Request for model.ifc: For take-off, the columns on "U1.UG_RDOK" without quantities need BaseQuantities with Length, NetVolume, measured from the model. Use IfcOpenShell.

First a look at what the model holds.

```python
import ifcopenshell
import ifcopenshell.util.element
import ifcopenshell.util.unit

model = ifcopenshell.open("model.ifc")
print(model.schema)
for unit_type in ("LENGTHUNIT", "AREAUNIT", "VOLUMEUNIT"):
    print(unit_type, ifcopenshell.util.unit.calculate_unit_scale(model, unit_type))
storey = next(s for s in model.by_type("IfcBuildingStorey") if s.Name == "U1.UG_RDOK")
columns = [e for e in ifcopenshell.util.element.get_decomposition(storey) if e.is_a("IfcColumn")]
for e in sorted(columns, key=lambda e: e.id()):
    print(e.id(), e.is_a(), e.Name, list(ifcopenshell.util.element.get_psets(e, qtos_only=True)), sep=" | ")
```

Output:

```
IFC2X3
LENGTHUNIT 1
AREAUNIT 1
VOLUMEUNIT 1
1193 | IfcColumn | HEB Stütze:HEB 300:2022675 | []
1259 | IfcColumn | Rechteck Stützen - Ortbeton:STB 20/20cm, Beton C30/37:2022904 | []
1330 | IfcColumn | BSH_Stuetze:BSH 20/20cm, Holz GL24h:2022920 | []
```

```python
import ifcopenshell
import ifcopenshell.api.pset
import ifcopenshell.geom
import ifcopenshell.util.element
import ifcopenshell.util.shape
import ifcopenshell.util.unit

model = ifcopenshell.open("model.ifc")
unit_scale = ifcopenshell.util.unit.calculate_unit_scale(model)
volume_scale = ifcopenshell.util.unit.calculate_unit_scale(model, "VOLUMEUNIT")
settings = ifcopenshell.geom.settings()

storey = next(s for s in model.by_type("IfcBuildingStorey") if s.Name == "U1.UG_RDOK")
columns = [e for e in ifcopenshell.util.element.get_decomposition(storey) if e.is_a("IfcColumn")]

for e in sorted(columns, key=lambda e: e.id()):
    if ifcopenshell.util.element.get_psets(e, qtos_only=True, should_inherit=False):
        continue
    # Geometry comes back in metres, in the element's own axes.
    shape = ifcopenshell.geom.create_shape(settings, e)
    values = {
        "Length": ifcopenshell.util.shape.get_z(shape.geometry) / unit_scale,
        "NetVolume": ifcopenshell.util.shape.get_volume(shape.geometry) / volume_scale,
    }
    qto = ifcopenshell.api.pset.add_qto(model, product=e, name="BaseQuantities")
    ifcopenshell.api.pset.edit_qto(model, qto=qto, properties=values)
    print(e.id(), {k: round(v, 3) for k, v in values.items()})

model.write("model_rev.ifc")
```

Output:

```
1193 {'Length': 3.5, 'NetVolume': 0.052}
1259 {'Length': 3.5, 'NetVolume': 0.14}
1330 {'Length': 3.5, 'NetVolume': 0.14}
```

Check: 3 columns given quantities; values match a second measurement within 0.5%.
